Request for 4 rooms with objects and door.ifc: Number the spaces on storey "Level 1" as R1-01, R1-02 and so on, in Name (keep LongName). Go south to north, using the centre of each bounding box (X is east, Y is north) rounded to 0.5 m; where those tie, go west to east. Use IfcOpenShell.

First a look at what the model holds.

```python
import ifcopenshell
import ifcopenshell.util.element
import ifcopenshell.util.placement

model = ifcopenshell.open("4 rooms with objects and door.ifc")
print(model.schema)
storey = next(s for s in model.by_type("IfcBuildingStorey") if s.Name == "Level 1")
spaces = [e for e in ifcopenshell.util.element.get_decomposition(storey) if e.is_a("IfcSpace")]
for e in sorted(spaces, key=lambda e: e.id()):
    origin = ifcopenshell.util.placement.get_local_placement(e.ObjectPlacement)[:3, 3]
    print(e.id(), e.Name, e.LongName, origin.round(2) + 0.0, sep=" | ")
```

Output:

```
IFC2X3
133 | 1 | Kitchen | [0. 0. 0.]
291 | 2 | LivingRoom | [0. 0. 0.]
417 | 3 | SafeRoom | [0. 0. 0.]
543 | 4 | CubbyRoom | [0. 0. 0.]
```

```python
import ifcopenshell
import ifcopenshell.geom
import ifcopenshell.util.element
import ifcopenshell.util.shape

model = ifcopenshell.open("4 rooms with objects and door.ifc")
settings = ifcopenshell.geom.settings()
settings.set("use-world-coords", True)


def centre(element):
    shape = ifcopenshell.geom.create_shape(settings, element)
    return ifcopenshell.util.shape.get_bbox_centroid(shape.geometry)


storey = next(s for s in model.by_type("IfcBuildingStorey") if s.Name == "Level 1")
spaces = [e for e in ifcopenshell.util.element.get_decomposition(storey) if e.is_a("IfcSpace")]

# Insertion points can sit at a corner or the storey origin, so sort by the geometry (in metres).
centres = {e: centre(e) for e in spaces}
spaces.sort(key=lambda e: (round(centres[e][1] / 0.5), centres[e][0]))

for i, e in enumerate(spaces, start=1):
    number = f"R1-{i:02d}"
    e.Name = number
    print(e.id(), number)

model.write("4 rooms with objects and door_rev.ifc")
```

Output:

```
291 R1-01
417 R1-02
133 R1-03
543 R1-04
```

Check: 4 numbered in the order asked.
